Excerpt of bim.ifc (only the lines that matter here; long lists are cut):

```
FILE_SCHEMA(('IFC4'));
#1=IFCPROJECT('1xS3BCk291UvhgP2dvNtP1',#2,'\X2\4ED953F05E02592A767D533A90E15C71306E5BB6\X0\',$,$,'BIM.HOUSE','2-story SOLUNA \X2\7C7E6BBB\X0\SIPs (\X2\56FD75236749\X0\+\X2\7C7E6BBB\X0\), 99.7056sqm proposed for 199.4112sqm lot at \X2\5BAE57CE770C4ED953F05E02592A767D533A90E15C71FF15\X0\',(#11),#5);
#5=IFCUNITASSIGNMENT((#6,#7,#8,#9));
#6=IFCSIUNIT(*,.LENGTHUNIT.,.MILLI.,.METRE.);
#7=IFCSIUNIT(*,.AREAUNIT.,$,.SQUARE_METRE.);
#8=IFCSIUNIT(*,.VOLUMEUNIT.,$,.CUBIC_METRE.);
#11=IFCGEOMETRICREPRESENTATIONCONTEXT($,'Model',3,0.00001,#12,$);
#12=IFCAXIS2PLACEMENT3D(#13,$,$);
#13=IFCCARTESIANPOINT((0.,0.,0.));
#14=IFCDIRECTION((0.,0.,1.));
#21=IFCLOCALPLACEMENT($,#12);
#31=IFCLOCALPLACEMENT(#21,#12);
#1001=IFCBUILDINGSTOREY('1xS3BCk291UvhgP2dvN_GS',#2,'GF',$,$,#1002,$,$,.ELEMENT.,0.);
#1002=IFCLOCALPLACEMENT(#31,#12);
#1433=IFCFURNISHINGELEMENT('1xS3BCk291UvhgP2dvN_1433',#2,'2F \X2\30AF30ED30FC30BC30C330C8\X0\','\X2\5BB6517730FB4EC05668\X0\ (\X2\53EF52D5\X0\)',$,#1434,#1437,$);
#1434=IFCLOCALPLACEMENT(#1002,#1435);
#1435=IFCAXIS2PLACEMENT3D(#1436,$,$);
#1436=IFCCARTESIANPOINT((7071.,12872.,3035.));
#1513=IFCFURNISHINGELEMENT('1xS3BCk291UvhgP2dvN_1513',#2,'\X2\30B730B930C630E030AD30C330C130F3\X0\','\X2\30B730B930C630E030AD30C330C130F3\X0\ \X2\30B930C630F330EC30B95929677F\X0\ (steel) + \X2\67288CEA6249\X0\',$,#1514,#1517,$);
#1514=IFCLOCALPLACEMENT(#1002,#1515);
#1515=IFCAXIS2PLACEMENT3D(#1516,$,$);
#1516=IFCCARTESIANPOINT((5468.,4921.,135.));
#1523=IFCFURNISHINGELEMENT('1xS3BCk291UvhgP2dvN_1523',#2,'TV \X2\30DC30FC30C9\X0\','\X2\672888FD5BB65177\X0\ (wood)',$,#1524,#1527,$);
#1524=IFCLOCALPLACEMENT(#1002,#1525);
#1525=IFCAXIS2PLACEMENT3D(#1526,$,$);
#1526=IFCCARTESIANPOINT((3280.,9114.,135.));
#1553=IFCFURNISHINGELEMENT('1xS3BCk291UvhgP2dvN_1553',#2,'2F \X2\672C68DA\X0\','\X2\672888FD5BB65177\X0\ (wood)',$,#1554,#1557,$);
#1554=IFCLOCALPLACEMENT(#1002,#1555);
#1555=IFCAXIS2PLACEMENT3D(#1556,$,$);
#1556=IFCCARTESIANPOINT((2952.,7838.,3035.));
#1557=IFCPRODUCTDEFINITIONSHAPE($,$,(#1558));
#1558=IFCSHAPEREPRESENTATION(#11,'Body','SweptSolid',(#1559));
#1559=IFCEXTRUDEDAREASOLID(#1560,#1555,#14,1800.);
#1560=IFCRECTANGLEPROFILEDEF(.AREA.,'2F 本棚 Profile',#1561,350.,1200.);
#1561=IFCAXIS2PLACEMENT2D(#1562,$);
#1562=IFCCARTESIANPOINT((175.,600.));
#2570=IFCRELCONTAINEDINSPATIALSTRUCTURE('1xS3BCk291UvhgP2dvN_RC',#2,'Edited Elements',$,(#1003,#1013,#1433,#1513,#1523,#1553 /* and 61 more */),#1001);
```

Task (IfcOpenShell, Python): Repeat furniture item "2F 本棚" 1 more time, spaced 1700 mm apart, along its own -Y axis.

```python
import ifcopenshell
import ifcopenshell.api.geometry
import ifcopenshell.api.root
import ifcopenshell.util.element
import ifcopenshell.util.placement

model = ifcopenshell.open("bim.ifc")


def reuse_history(source, copy):
    """copy_class also copies each property set's owner history, people and application; keep the originals."""
    for rel in copy.IsDefinedBy:
        if rel.is_a("IfcRelDefinesByProperties") and (history := rel.RelatingPropertyDefinition.OwnerHistory):
            rel.RelatingPropertyDefinition.OwnerHistory = source.OwnerHistory
            ifcopenshell.util.element.remove_deep2(model, history)


source = model.by_id(1553)
base = ifcopenshell.util.placement.get_local_placement(source.ObjectPlacement)
step = -base[:3, 1] * 1700.0

for i in range(1, 2):
    copy = ifcopenshell.api.root.copy_class(model, product=source)
    copy.Representation = ifcopenshell.util.element.copy_deep(
        model, source.Representation, exclude=["IfcGeometricRepresentationContext", "IfcRepresentationMap"]
    )
    reuse_history(source, copy)
    matrix = base.copy()
    matrix[:3, 3] += i * step
    print("added at", matrix[:3, 3].round(3) + 0.0)
    ifcopenshell.api.geometry.edit_object_placement(model, product=copy, matrix=matrix, is_si=False)

model.write("bim_edited.ifc")
```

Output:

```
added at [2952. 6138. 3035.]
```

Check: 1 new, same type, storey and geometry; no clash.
